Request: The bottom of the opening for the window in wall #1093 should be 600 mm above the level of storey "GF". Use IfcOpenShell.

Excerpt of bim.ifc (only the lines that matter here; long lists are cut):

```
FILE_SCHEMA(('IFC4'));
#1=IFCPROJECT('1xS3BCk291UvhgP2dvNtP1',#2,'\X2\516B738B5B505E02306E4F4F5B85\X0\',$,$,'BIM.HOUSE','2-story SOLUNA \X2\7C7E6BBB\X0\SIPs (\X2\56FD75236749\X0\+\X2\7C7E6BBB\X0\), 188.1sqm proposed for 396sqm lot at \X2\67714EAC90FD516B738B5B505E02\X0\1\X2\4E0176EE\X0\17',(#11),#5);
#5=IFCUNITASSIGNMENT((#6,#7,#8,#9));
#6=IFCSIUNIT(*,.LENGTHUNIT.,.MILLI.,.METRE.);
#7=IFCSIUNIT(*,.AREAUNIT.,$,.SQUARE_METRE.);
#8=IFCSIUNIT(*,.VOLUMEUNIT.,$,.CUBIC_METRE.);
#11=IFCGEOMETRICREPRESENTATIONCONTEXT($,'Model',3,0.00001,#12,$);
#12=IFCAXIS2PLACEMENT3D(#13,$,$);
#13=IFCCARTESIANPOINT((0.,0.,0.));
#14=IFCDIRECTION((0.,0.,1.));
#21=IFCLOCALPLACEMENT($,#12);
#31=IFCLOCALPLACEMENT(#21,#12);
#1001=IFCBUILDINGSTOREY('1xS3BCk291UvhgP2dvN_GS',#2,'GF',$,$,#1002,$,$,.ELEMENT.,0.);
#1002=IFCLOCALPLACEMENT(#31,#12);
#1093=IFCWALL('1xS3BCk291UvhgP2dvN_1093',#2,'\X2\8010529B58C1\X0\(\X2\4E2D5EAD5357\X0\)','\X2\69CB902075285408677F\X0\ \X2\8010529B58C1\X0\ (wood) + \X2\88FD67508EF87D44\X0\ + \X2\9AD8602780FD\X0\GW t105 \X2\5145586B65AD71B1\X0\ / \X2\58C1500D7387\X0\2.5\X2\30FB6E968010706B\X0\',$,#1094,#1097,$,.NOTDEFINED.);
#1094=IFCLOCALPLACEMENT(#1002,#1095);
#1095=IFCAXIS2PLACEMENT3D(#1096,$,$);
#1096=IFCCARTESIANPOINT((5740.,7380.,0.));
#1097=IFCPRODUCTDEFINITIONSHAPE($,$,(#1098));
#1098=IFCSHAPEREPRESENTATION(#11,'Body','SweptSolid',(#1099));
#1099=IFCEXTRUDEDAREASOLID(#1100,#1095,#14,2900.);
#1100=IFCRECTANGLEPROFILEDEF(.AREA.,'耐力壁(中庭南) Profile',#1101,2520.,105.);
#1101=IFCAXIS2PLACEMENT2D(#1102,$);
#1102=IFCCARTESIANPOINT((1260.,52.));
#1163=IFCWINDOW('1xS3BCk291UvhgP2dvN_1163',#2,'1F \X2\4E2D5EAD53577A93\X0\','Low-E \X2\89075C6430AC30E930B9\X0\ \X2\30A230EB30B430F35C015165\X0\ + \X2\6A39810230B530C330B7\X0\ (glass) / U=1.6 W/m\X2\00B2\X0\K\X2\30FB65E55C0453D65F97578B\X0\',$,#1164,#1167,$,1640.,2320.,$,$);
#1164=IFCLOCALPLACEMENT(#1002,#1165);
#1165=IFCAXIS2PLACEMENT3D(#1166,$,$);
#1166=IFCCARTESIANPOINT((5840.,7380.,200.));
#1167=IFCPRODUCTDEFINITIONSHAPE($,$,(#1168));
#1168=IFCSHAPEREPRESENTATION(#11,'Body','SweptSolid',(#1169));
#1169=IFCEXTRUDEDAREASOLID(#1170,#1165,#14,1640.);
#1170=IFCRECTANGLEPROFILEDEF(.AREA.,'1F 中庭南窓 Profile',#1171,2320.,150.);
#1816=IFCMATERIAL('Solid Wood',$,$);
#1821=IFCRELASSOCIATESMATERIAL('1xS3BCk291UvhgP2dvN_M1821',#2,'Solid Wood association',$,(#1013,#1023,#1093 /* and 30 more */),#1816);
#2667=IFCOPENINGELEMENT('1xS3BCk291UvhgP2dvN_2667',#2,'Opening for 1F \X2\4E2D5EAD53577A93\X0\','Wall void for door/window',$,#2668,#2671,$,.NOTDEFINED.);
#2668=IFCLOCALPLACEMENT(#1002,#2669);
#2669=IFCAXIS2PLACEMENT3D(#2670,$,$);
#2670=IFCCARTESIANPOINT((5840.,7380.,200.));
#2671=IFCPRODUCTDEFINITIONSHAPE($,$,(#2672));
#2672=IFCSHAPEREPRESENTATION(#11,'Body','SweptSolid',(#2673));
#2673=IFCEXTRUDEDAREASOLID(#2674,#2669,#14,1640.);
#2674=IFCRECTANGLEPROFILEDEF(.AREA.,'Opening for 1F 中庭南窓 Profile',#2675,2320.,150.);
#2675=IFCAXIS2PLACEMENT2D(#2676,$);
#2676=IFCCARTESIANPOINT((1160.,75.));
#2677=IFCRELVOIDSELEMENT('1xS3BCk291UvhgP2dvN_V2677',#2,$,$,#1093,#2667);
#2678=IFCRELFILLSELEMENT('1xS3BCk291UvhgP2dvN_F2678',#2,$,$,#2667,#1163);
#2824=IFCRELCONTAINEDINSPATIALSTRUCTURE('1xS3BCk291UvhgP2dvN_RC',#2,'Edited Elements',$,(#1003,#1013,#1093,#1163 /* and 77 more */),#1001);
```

```python
import numpy as np
import ifcopenshell
import ifcopenshell.api.geometry
import ifcopenshell.geom
import ifcopenshell.util.element
import ifcopenshell.util.placement
import ifcopenshell.util.shape
import ifcopenshell.util.unit

model = ifcopenshell.open("bim.ifc")
unit_scale = ifcopenshell.util.unit.calculate_unit_scale(model)

window = model.by_guid("1xS3BCk291UvhgP2dvN_1163")
opening = window.FillsVoids[0].RelatingOpeningElement
storey = ifcopenshell.util.element.get_container(window, ifc_class="IfcBuildingStorey")
level = ifcopenshell.util.placement.get_local_placement(storey.ObjectPlacement)[2, 3]

# The opening's origin need not be at the sill, so measure its lowest point.
shape = ifcopenshell.geom.create_shape(ifcopenshell.geom.settings(), opening)
bottom = ifcopenshell.util.shape.get_shape_bottom_elevation(shape, shape.geometry) / unit_scale
dz = level + 0.6 / unit_scale - bottom

shift = np.array([0.0, 0.0, dz])
# The window is not placed relative to its opening, so move both.
for product in (opening, window):
    matrix = ifcopenshell.util.placement.get_local_placement(product.ObjectPlacement)
    matrix[:3, 3] += shift
    ifcopenshell.api.geometry.edit_object_placement(model, product=product, matrix=matrix, is_si=False)

print(f"moved by {dz * unit_scale:+.3f} m")

model.write("bim_v2.ifc")
```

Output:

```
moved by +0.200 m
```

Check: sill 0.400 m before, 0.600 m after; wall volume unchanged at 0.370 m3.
